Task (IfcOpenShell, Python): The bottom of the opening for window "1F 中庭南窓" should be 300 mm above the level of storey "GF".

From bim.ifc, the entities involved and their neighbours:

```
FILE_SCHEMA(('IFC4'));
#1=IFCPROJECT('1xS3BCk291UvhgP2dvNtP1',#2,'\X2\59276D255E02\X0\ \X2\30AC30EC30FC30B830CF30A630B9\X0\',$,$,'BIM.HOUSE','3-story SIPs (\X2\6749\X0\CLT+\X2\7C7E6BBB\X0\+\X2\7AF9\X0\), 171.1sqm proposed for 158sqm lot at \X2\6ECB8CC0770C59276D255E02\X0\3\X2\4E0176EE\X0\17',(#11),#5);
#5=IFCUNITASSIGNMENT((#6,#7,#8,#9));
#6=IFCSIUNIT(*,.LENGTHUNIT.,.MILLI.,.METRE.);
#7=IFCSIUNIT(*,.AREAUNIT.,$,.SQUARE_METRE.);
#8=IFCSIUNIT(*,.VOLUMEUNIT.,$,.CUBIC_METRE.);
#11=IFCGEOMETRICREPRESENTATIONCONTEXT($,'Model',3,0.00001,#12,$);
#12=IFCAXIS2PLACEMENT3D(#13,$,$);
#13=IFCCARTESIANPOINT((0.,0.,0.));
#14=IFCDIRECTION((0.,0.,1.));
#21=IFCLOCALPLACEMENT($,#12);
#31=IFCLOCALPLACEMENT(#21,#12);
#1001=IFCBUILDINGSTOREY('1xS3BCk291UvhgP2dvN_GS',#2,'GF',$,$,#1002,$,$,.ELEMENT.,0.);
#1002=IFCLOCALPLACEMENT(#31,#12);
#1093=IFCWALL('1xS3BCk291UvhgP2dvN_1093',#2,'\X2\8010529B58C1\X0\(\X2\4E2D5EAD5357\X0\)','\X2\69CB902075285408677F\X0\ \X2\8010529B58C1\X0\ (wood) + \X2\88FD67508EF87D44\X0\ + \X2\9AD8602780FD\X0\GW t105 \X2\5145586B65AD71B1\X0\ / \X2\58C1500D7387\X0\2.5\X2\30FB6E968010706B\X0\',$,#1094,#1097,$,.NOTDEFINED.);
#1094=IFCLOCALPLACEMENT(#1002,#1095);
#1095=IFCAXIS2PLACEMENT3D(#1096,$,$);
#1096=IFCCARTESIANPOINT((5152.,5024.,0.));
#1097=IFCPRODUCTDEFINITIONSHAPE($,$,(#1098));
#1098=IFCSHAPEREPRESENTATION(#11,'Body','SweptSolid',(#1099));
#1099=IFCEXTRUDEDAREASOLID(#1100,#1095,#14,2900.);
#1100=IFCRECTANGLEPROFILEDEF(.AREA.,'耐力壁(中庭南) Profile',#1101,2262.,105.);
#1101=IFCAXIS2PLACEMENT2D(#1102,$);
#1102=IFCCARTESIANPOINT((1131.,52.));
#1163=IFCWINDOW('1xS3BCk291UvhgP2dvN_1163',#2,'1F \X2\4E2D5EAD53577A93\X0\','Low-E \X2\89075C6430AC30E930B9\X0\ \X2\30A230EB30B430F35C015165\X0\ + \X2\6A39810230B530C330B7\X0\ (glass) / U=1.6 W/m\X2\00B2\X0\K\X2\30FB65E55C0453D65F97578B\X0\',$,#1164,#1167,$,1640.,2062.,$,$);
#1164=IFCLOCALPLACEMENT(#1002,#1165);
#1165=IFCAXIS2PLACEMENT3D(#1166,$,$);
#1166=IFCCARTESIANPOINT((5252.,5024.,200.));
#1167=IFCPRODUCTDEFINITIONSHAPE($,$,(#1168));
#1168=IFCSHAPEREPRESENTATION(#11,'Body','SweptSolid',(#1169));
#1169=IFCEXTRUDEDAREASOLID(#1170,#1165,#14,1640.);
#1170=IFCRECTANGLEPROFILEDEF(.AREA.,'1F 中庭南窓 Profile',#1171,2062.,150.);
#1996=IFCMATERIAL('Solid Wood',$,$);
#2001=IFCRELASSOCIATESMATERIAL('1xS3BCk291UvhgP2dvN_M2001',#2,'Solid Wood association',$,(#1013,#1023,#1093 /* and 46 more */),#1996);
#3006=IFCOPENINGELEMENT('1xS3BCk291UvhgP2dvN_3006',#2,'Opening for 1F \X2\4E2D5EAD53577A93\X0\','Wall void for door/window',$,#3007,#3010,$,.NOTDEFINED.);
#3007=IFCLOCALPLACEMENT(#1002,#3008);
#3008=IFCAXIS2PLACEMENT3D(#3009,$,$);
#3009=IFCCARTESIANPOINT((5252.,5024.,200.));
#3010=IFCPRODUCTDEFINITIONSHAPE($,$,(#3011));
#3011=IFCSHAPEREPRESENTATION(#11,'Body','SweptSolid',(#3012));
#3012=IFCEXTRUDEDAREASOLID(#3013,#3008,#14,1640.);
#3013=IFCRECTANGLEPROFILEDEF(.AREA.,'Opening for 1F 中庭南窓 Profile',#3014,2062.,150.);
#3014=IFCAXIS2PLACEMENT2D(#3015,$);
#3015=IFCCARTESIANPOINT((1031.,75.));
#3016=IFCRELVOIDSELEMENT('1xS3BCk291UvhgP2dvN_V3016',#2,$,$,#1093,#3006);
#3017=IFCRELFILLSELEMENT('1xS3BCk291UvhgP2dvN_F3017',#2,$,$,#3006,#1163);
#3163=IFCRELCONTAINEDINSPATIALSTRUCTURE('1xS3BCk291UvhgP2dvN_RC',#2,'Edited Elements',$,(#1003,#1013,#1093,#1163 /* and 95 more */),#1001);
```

```python
import numpy as np
import ifcopenshell
import ifcopenshell.api.geometry
import ifcopenshell.geom
import ifcopenshell.util.element
import ifcopenshell.util.placement
import ifcopenshell.util.shape
import ifcopenshell.util.unit

model = ifcopenshell.open("bim.ifc")
unit_scale = ifcopenshell.util.unit.calculate_unit_scale(model)

window = model.by_guid("1xS3BCk291UvhgP2dvN_1163")
opening = window.FillsVoids[0].RelatingOpeningElement
storey = ifcopenshell.util.element.get_container(window, ifc_class="IfcBuildingStorey")
level = ifcopenshell.util.placement.get_local_placement(storey.ObjectPlacement)[2, 3]

# The opening's origin need not be at the sill, so measure its lowest point.
shape = ifcopenshell.geom.create_shape(ifcopenshell.geom.settings(), opening)
bottom = ifcopenshell.util.shape.get_shape_bottom_elevation(shape, shape.geometry) / unit_scale
dz = level + 0.3 / unit_scale - bottom

shift = np.array([0.0, 0.0, dz])
# The window is not placed relative to its opening, so move both.
for product in (opening, window):
    matrix = ifcopenshell.util.placement.get_local_placement(product.ObjectPlacement)
    matrix[:3, 3] += shift
    ifcopenshell.api.geometry.edit_object_placement(model, product=product, matrix=matrix, is_si=False)

print(f"moved by {dz * unit_scale:+.3f} m")

model.write("bim_v2.ifc")
```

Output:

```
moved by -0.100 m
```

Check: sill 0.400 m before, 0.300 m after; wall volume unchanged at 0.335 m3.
